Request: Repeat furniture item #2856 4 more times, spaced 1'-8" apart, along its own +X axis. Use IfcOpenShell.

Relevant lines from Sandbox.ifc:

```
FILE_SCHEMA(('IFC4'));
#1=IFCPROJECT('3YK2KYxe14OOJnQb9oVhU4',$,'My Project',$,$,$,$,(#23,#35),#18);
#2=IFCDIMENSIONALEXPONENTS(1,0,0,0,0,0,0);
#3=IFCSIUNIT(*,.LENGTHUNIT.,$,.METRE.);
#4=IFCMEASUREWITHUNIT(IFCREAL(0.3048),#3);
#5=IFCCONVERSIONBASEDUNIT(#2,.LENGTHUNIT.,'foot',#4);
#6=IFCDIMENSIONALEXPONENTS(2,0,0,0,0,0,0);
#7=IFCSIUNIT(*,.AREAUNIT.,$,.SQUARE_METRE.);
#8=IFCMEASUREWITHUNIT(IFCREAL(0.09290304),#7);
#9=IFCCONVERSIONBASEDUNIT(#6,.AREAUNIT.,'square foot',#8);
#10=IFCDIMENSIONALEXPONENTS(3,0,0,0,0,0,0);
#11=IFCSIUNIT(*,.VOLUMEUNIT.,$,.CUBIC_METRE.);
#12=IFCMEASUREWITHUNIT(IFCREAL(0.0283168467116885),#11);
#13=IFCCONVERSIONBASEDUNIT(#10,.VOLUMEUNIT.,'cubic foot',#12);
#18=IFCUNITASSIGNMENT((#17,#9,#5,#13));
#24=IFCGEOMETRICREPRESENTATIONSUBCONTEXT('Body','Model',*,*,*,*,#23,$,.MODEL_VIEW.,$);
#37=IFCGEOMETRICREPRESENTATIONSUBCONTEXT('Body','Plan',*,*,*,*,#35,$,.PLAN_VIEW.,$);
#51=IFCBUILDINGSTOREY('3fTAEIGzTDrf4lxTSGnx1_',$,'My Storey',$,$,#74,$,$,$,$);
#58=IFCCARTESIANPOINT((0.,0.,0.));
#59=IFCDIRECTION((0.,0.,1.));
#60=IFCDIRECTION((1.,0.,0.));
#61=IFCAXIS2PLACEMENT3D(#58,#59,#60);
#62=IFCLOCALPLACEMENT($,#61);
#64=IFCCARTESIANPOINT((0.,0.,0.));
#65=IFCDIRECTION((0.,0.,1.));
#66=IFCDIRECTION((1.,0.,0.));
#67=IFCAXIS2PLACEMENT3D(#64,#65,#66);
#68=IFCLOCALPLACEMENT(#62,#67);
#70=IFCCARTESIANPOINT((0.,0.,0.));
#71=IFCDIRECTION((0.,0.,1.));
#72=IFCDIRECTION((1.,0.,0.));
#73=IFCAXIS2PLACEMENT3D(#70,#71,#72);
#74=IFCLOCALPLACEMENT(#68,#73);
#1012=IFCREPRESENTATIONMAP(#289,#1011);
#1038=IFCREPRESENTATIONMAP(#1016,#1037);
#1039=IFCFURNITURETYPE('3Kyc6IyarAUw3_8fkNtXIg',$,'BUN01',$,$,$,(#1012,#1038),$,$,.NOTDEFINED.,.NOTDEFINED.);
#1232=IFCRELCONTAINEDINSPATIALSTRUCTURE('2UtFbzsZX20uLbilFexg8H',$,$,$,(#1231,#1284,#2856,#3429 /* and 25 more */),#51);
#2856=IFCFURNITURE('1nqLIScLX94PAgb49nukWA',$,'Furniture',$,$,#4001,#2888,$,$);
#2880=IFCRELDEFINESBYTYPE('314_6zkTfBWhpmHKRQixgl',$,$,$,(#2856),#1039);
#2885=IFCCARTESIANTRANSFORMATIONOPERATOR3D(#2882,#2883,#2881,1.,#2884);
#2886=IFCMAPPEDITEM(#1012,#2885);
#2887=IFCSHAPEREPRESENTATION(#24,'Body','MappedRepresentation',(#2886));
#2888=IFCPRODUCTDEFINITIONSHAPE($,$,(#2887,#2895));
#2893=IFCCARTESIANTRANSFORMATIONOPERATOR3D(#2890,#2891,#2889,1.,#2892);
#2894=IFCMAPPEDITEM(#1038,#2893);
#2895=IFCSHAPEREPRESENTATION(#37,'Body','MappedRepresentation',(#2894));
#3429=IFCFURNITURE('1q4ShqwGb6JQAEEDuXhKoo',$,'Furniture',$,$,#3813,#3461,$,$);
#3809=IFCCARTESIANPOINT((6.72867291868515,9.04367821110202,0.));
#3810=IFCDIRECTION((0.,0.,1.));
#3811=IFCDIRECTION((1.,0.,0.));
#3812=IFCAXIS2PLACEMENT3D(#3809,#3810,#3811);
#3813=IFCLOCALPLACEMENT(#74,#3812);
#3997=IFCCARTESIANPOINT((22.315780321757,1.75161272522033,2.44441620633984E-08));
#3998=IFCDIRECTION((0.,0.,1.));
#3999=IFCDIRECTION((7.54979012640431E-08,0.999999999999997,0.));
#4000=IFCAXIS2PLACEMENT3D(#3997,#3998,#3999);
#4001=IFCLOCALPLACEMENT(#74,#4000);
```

```python
import ifcopenshell
import ifcopenshell.api.geometry
import ifcopenshell.api.root
import ifcopenshell.util.element
import ifcopenshell.util.placement
import ifcopenshell.util.unit

model = ifcopenshell.open("Sandbox.ifc")
unit_scale = ifcopenshell.util.unit.calculate_unit_scale(model)

source = model.by_guid("1nqLIScLX94PAgb49nukWA")
base = ifcopenshell.util.placement.get_local_placement(source.ObjectPlacement)
step = base[:3, 0] * 20 * 0.0254 / unit_scale

for i in range(1, 5):
    copy = ifcopenshell.api.root.copy_class(model, product=source)
    copy.Representation = ifcopenshell.util.element.copy_deep(
        model, source.Representation, exclude=["IfcGeometricRepresentationContext", "IfcRepresentationMap"]
    )
    matrix = base.copy()
    matrix[:3, 3] += i * step
    print("added at", matrix[:3, 3].round(3) + 0.0)
    ifcopenshell.api.geometry.edit_object_placement(model, product=copy, matrix=matrix, is_si=False)

model.write("Sandbox_updated.ifc")
```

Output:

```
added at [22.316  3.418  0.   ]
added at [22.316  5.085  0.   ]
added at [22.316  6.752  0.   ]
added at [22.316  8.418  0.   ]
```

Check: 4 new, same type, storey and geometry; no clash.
